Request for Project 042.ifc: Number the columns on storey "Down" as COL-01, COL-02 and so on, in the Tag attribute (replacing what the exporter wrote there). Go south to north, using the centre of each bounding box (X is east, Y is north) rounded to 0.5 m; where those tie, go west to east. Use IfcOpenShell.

First a look at what the model holds.

```python
import ifcopenshell
import ifcopenshell.util.element
import ifcopenshell.util.placement

model = ifcopenshell.open("Project 042.ifc")
print(model.schema)
storey = next(s for s in model.by_type("IfcBuildingStorey") if s.Name == "Down")
columns = [e for e in ifcopenshell.util.element.get_decomposition(storey) if e.is_a("IfcColumn")]
for e in sorted(columns, key=lambda e: e.id()):
    origin = ifcopenshell.util.placement.get_local_placement(e.ObjectPlacement)[:3, 3]
    print(e.id(), e.Tag, e.Name, origin.round(2) + 0.0, sep=" | ")
```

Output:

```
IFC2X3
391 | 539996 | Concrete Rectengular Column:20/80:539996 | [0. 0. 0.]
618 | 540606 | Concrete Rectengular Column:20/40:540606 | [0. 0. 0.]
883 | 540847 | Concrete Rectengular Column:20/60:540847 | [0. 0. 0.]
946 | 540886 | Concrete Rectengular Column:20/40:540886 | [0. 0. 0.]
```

```python
import ifcopenshell
import ifcopenshell.geom
import ifcopenshell.util.element
import ifcopenshell.util.shape

model = ifcopenshell.open("Project 042.ifc")
settings = ifcopenshell.geom.settings()
settings.set("use-world-coords", True)


def centre(element):
    shape = ifcopenshell.geom.create_shape(settings, element)
    return ifcopenshell.util.shape.get_bbox_centroid(shape.geometry)


storey = next(s for s in model.by_type("IfcBuildingStorey") if s.Name == "Down")
columns = [e for e in ifcopenshell.util.element.get_decomposition(storey) if e.is_a("IfcColumn")]

# Insertion points can sit at a corner or the storey origin, so sort by the geometry (in metres).
centres = {e: centre(e) for e in columns}
columns.sort(key=lambda e: (round(centres[e][1] / 0.5), centres[e][0]))

for i, e in enumerate(columns, start=1):
    number = f"COL-{i:02d}"
    e.Tag = number
    print(e.id(), number)

model.write("Project 042_updated.ifc")
```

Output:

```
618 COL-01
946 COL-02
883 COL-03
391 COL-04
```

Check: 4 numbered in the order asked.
